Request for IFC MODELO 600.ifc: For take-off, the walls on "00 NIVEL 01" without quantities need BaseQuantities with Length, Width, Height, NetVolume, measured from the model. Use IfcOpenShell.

First a look at what the model holds.

```python
import ifcopenshell
import ifcopenshell.util.element
import ifcopenshell.util.unit

model = ifcopenshell.open("IFC MODELO 600.ifc")
print(model.schema)
for unit_type in ("LENGTHUNIT", "AREAUNIT", "VOLUMEUNIT"):
    print(unit_type, ifcopenshell.util.unit.calculate_unit_scale(model, unit_type))
storey = next(s for s in model.by_type("IfcBuildingStorey") if s.Name == "00 NIVEL 01")
walls = [e for e in ifcopenshell.util.element.get_decomposition(storey) if e.is_a("IfcWall")]
for e in sorted(walls, key=lambda e: e.id()):
    print(e.id(), e.is_a(), e.Name, list(ifcopenshell.util.element.get_psets(e, qtos_only=True)), sep=" | ")
```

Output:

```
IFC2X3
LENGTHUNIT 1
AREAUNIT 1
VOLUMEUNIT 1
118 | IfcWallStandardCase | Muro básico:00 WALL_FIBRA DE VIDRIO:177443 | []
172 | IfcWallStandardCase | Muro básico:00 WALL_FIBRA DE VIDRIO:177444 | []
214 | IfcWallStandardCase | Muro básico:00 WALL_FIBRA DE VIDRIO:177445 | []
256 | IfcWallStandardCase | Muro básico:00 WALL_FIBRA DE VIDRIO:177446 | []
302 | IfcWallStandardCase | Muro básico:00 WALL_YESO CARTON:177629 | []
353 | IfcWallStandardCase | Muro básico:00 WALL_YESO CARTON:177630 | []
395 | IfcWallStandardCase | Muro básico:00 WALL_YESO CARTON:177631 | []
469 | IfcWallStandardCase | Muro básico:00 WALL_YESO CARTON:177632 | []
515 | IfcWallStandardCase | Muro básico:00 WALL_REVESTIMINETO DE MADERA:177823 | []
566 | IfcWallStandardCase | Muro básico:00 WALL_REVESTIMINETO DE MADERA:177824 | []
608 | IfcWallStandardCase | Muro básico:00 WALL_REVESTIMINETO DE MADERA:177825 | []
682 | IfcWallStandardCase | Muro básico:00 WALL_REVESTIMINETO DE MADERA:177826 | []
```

```python
import ifcopenshell
import ifcopenshell.api.pset
import ifcopenshell.geom
import ifcopenshell.util.element
import ifcopenshell.util.shape
import ifcopenshell.util.unit

model = ifcopenshell.open("IFC MODELO 600.ifc")
unit_scale = ifcopenshell.util.unit.calculate_unit_scale(model)
volume_scale = ifcopenshell.util.unit.calculate_unit_scale(model, "VOLUMEUNIT")
settings = ifcopenshell.geom.settings()

storey = next(s for s in model.by_type("IfcBuildingStorey") if s.Name == "00 NIVEL 01")
walls = [e for e in ifcopenshell.util.element.get_decomposition(storey) if e.is_a("IfcWall")]

for e in sorted(walls, key=lambda e: e.id()):
    if ifcopenshell.util.element.get_psets(e, qtos_only=True, should_inherit=False):
        continue
    # Geometry comes back in metres, in the element's own axes.
    shape = ifcopenshell.geom.create_shape(settings, e)
    values = {
        "Length": ifcopenshell.util.shape.get_x(shape.geometry) / unit_scale,
        "Width": ifcopenshell.util.shape.get_y(shape.geometry) / unit_scale,
        "Height": ifcopenshell.util.shape.get_z(shape.geometry) / unit_scale,
        "NetVolume": ifcopenshell.util.shape.get_volume(shape.geometry) / volume_scale,
    }
    qto = ifcopenshell.api.pset.add_qto(model, product=e, name="BaseQuantities")
    ifcopenshell.api.pset.edit_qto(model, qto=qto, properties=values)
    print(e.id(), {k: round(v, 3) for k, v in values.items()})

model.write("IFC MODELO 600_rev.ifc")
```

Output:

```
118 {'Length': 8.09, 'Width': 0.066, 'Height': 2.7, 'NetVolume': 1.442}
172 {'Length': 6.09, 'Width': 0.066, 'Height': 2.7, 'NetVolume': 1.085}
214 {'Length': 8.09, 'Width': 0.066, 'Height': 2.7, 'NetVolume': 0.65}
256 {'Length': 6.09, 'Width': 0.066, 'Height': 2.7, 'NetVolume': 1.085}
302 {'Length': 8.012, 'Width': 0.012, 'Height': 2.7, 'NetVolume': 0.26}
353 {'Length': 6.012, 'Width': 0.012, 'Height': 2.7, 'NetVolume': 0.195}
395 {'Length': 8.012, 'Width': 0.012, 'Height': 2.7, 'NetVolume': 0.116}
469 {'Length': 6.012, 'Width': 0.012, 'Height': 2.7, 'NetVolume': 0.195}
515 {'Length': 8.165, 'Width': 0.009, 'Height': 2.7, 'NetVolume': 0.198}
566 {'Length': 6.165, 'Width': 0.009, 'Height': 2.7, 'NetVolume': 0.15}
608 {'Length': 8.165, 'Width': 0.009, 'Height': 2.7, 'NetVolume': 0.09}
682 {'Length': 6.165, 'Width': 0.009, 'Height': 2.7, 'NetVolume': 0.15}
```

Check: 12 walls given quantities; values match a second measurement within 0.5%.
